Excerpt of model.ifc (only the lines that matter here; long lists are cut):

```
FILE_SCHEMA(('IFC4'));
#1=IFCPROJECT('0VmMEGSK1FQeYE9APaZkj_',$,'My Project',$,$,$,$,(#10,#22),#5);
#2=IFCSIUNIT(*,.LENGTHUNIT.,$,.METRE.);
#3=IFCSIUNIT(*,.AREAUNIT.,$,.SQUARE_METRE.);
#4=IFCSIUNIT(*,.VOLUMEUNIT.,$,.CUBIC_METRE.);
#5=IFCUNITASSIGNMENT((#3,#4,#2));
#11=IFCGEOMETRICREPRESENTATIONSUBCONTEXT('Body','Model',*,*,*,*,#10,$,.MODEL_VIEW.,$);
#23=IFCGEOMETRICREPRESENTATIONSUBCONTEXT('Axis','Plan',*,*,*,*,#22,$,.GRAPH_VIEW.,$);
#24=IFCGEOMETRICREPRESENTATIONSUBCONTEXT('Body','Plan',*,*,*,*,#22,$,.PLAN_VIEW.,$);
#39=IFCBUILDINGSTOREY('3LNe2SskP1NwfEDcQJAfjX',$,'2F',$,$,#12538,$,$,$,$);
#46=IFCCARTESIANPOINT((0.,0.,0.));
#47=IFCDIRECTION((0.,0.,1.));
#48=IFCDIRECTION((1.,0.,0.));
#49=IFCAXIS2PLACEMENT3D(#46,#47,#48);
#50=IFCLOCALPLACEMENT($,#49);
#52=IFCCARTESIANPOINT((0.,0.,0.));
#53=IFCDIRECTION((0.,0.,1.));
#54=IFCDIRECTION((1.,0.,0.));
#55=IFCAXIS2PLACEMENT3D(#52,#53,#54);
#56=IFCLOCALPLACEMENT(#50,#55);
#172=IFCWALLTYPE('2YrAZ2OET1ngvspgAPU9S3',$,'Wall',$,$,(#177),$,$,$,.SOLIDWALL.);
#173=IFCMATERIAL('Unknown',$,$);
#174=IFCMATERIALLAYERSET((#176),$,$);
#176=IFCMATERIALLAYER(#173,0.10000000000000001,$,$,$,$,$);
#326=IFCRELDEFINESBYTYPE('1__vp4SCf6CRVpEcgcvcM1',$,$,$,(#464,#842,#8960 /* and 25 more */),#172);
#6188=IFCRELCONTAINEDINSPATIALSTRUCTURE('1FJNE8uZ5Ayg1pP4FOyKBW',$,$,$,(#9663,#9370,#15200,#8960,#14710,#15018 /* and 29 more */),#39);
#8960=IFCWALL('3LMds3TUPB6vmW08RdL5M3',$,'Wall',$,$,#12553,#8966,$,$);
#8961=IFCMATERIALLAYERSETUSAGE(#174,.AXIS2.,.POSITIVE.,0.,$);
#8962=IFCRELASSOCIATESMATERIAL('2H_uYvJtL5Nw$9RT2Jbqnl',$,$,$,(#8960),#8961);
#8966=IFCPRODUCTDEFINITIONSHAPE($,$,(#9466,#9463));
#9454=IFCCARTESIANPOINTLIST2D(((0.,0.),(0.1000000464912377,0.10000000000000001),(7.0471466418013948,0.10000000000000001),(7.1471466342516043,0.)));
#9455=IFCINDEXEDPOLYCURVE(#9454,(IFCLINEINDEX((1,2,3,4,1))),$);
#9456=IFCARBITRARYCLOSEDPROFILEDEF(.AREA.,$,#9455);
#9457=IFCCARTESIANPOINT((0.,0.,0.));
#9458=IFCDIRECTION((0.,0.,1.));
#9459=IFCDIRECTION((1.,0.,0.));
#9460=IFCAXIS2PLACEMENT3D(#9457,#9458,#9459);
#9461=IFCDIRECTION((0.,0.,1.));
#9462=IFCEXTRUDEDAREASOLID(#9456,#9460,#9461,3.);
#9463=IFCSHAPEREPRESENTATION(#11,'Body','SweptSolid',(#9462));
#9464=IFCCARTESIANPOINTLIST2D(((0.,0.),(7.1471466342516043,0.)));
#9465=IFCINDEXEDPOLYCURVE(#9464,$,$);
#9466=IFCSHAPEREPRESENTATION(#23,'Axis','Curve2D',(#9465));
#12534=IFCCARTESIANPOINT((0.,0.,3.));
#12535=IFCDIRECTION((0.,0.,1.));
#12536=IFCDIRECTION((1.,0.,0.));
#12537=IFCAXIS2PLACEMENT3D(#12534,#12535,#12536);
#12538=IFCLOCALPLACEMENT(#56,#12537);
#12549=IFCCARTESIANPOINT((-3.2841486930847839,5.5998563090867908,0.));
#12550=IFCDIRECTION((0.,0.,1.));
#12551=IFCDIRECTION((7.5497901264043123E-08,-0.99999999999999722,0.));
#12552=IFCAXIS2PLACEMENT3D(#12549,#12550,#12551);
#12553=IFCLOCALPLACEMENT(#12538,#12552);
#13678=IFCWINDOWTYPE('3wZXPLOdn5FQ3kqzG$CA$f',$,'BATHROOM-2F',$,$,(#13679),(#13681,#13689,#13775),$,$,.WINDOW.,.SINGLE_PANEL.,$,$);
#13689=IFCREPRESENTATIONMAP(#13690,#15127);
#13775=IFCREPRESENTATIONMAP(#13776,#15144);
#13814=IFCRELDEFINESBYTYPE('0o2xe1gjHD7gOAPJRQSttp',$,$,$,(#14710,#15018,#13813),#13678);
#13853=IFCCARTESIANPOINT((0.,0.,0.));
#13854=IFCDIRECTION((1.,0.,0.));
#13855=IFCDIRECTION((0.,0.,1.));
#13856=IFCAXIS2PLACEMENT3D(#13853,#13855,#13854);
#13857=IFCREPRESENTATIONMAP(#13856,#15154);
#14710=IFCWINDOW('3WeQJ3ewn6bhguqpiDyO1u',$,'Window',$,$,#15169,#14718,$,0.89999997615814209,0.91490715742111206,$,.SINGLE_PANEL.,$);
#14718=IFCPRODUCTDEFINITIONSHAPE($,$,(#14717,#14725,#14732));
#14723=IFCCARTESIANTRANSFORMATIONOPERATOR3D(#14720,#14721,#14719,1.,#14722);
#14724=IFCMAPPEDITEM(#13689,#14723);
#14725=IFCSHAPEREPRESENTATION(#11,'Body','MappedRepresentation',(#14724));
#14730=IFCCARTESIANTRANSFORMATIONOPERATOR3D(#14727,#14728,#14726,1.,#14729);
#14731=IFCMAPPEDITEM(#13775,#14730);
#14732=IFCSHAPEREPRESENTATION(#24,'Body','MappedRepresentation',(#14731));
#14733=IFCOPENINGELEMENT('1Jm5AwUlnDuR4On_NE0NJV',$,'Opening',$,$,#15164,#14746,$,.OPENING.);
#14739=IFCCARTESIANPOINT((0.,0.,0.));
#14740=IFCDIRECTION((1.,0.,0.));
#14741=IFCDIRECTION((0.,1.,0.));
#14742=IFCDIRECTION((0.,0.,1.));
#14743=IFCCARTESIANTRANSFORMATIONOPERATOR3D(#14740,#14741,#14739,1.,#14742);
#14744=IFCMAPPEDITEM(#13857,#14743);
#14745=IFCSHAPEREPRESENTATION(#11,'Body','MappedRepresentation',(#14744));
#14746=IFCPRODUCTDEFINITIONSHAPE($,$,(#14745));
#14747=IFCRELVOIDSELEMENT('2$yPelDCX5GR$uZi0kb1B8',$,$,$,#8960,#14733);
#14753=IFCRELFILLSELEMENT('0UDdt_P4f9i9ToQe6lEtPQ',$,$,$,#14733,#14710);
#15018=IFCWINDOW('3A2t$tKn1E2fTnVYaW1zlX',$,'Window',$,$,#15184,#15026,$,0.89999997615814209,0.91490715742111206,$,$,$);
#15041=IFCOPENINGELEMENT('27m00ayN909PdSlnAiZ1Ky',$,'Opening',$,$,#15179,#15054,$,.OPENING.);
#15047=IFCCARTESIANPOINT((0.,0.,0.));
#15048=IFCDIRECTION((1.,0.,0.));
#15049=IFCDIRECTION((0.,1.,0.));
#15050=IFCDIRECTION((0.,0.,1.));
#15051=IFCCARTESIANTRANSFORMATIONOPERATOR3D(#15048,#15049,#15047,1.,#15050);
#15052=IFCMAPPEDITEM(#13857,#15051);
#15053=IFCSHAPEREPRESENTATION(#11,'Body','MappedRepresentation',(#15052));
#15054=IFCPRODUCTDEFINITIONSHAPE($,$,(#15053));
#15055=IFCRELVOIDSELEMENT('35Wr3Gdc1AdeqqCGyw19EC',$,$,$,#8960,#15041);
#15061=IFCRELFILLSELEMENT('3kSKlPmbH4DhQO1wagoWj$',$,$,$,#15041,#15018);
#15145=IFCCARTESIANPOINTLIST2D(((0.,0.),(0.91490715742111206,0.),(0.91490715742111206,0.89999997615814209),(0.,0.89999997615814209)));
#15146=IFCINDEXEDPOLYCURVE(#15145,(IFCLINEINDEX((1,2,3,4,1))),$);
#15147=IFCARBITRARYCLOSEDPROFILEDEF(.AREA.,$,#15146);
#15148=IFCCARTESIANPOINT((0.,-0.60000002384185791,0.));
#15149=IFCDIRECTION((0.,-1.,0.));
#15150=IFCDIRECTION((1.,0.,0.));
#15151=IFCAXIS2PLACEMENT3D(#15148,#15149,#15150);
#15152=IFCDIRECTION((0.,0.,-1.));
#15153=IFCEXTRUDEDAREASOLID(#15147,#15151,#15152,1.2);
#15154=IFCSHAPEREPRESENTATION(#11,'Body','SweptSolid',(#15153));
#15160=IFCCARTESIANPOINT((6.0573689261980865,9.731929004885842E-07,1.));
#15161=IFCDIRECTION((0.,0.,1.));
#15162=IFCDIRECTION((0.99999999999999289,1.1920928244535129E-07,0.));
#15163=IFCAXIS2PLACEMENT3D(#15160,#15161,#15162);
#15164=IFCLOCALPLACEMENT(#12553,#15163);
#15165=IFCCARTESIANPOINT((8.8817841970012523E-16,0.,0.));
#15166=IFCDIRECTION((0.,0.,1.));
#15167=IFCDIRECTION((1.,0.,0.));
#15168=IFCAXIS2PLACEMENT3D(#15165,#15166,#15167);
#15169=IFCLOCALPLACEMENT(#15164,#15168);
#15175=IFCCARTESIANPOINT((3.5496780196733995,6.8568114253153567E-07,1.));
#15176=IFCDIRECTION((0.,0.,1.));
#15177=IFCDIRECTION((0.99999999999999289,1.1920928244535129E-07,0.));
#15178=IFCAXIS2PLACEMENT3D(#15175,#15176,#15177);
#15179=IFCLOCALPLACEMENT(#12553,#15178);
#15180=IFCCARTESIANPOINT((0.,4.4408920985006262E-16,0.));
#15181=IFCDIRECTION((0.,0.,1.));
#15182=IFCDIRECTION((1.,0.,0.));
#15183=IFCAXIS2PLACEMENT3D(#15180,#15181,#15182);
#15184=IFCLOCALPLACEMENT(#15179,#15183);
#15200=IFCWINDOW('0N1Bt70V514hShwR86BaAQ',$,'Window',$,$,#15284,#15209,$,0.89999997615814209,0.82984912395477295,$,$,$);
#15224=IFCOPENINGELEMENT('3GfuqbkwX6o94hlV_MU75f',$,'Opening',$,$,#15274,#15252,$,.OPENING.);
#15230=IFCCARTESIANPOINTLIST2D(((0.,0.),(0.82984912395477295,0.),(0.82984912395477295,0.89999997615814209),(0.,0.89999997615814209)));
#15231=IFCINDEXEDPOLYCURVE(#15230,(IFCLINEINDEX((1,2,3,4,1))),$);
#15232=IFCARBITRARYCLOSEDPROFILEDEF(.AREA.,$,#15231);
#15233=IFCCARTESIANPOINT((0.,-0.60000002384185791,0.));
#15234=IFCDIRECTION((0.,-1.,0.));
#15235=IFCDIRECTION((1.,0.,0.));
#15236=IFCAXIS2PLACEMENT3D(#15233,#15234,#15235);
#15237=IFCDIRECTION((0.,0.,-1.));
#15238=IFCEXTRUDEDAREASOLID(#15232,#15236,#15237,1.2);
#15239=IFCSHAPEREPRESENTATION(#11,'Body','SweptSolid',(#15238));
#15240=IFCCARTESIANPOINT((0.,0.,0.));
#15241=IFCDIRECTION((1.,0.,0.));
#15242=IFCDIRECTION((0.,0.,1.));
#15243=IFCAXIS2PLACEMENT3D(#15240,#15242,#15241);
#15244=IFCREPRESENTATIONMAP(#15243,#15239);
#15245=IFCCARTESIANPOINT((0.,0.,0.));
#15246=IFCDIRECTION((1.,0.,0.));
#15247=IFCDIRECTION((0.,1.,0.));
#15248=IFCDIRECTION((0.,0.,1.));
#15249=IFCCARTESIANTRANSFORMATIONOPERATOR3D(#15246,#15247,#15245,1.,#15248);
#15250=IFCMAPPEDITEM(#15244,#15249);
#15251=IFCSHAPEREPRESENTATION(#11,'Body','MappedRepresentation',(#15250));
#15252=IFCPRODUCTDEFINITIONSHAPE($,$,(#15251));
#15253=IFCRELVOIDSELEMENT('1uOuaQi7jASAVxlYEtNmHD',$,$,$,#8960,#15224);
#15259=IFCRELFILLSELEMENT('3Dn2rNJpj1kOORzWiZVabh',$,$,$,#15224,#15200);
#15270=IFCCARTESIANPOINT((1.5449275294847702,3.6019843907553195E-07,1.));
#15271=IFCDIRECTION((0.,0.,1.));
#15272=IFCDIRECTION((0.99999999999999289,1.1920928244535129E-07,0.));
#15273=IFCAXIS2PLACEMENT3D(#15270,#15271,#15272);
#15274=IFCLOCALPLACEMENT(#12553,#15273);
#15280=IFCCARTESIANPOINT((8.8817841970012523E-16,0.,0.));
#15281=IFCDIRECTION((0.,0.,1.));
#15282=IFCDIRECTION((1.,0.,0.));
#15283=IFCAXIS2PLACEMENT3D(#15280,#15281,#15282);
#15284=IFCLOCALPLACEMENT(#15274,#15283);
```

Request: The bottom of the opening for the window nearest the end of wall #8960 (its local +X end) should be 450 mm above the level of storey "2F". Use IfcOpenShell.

```python
import numpy as np
import ifcopenshell
import ifcopenshell.api.geometry
import ifcopenshell.geom
import ifcopenshell.util.element
import ifcopenshell.util.placement
import ifcopenshell.util.shape
import ifcopenshell.util.unit

model = ifcopenshell.open("model.ifc")
unit_scale = ifcopenshell.util.unit.calculate_unit_scale(model)

window = model.by_guid("3WeQJ3ewn6bhguqpiDyO1u")
opening = window.FillsVoids[0].RelatingOpeningElement
storey = ifcopenshell.util.element.get_container(window, ifc_class="IfcBuildingStorey")
level = ifcopenshell.util.placement.get_local_placement(storey.ObjectPlacement)[2, 3]

# The opening's origin need not be at the sill, so measure its lowest point.
shape = ifcopenshell.geom.create_shape(ifcopenshell.geom.settings(), opening)
bottom = ifcopenshell.util.shape.get_shape_bottom_elevation(shape, shape.geometry) / unit_scale
dz = level + 0.45 - bottom

shift = np.array([0.0, 0.0, dz])
# The window is placed relative to its opening, so it follows when the opening moves.
matrix = ifcopenshell.util.placement.get_local_placement(opening.ObjectPlacement)
matrix[:3, 3] += shift
ifcopenshell.api.geometry.edit_object_placement(
    model, product=opening, matrix=matrix, is_si=False, should_transform_children=True
)

print(f"moved by {dz * unit_scale:+.3f} m")

model.write("model_rev.ifc")
```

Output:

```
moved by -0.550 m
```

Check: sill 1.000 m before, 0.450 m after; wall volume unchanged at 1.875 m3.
